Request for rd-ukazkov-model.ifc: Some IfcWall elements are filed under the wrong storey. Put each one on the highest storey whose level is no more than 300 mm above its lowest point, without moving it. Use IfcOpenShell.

First a look at what the model holds.

```python
import ifcopenshell
import ifcopenshell.util.element
import ifcopenshell.util.placement

model = ifcopenshell.open("rd-ukazkov-model.ifc")
print(model.schema)
for storey in model.by_type("IfcBuildingStorey"):
    level = ifcopenshell.util.placement.get_storey_elevation(storey)
    count = sum(e.is_a("IfcWall") for e in ifcopenshell.util.element.get_contained(storey))
    print(storey.id(), storey.Name, round(level, 3), count, sep=" | ")
```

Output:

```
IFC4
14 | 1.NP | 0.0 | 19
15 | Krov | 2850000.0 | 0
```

```python
import ifcopenshell
import ifcopenshell.api.spatial
import ifcopenshell.geom
import ifcopenshell.util.element
import ifcopenshell.util.placement
import ifcopenshell.util.shape
import ifcopenshell.util.unit

model = ifcopenshell.open("rd-ukazkov-model.ifc")
unit_scale = ifcopenshell.util.unit.calculate_unit_scale(model)
settings = ifcopenshell.geom.settings()

levels = sorted(
    ((ifcopenshell.util.placement.get_storey_elevation(s) * unit_scale, s) for s in model.by_type("IfcBuildingStorey")),
    key=lambda pair: pair[0],
)

for e in model.by_type("IfcWall"):
    current = e.ContainedInStructure[0].RelatingStructure if e.ContainedInStructure else None
    if current is None or not current.is_a("IfcBuildingStorey"):
        continue
    shape = ifcopenshell.geom.create_shape(settings, e)
    bottom = ifcopenshell.util.shape.get_shape_bottom_elevation(shape, shape.geometry)
    below = [s for level, s in levels if level <= bottom + 0.3]
    storey = below[-1] if below else levels[0][1]
    if storey != current:
        # assign_container keeps the world position.
        ifcopenshell.api.spatial.assign_container(model, products=[e], relating_structure=storey)
        print(e.id(), current.Name, "->", storey.Name)

model.write("rd-ukazkov-model_rev.ifc")
```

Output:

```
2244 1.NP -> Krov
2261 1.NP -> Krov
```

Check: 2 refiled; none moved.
